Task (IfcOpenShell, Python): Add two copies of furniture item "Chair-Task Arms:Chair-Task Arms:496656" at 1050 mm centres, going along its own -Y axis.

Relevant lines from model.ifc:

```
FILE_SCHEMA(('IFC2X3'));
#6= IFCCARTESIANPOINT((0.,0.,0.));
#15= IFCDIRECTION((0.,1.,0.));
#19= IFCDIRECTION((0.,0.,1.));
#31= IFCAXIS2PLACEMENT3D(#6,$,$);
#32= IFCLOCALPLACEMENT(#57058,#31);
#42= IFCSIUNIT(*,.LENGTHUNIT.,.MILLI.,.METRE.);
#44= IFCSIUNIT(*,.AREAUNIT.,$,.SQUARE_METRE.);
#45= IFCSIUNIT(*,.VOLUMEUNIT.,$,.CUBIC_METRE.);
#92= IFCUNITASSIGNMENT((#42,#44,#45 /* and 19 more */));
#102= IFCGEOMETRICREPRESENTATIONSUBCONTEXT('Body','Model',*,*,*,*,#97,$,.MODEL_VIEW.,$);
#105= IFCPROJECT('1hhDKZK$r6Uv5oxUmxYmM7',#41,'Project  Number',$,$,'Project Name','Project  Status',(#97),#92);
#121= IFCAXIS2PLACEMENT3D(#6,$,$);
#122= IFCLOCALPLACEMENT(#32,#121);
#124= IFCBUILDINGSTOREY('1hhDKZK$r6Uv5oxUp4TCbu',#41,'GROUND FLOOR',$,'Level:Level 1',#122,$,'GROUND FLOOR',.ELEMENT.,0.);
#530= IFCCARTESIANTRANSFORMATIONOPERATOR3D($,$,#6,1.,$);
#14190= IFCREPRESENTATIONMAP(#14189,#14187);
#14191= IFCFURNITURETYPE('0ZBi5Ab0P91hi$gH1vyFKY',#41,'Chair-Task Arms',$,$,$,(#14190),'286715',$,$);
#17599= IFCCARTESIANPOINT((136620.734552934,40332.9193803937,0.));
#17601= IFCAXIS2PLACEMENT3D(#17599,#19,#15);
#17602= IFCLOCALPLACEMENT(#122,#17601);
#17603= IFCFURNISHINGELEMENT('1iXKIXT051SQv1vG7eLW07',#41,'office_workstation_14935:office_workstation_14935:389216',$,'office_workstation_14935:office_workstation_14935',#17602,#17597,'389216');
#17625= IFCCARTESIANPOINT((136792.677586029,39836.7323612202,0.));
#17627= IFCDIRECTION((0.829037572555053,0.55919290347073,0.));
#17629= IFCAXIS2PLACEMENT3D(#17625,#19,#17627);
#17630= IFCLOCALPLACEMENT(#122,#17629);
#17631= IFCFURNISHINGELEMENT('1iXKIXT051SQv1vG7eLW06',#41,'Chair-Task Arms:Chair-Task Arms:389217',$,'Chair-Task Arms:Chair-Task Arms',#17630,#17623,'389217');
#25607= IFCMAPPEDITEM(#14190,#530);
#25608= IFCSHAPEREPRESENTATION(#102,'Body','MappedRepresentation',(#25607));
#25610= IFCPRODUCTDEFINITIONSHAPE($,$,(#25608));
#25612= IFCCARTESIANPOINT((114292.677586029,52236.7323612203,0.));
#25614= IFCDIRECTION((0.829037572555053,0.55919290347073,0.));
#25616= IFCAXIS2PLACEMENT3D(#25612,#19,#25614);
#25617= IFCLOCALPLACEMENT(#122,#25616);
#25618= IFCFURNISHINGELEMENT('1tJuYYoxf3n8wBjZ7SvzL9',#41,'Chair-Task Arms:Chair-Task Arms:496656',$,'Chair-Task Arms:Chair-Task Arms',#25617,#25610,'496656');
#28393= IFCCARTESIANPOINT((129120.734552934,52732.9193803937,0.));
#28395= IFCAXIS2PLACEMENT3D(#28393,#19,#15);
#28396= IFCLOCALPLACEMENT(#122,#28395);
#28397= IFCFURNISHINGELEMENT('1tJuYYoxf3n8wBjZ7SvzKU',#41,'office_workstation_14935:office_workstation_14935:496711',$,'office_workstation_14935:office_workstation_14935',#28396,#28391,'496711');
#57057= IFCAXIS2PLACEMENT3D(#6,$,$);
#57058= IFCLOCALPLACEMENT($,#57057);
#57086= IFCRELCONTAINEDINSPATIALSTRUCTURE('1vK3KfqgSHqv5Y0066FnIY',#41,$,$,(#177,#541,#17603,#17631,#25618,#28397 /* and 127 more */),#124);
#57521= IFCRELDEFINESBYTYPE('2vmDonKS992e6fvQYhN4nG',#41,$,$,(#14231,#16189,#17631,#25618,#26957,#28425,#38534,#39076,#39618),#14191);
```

```python
import ifcopenshell
import ifcopenshell.api.geometry
import ifcopenshell.api.root
import ifcopenshell.util.element
import ifcopenshell.util.placement
import ifcopenshell.util.unit

model = ifcopenshell.open("model.ifc")
unit_scale = ifcopenshell.util.unit.calculate_unit_scale(model)


def reuse_history(source, copy):
    """copy_class also copies each property set's owner history, people and application; keep the originals."""
    for rel in copy.IsDefinedBy:
        if rel.is_a("IfcRelDefinesByProperties") and (history := rel.RelatingPropertyDefinition.OwnerHistory):
            rel.RelatingPropertyDefinition.OwnerHistory = source.OwnerHistory
            ifcopenshell.util.element.remove_deep2(model, history)


source = model.by_id(25618)
base = ifcopenshell.util.placement.get_local_placement(source.ObjectPlacement)
step = -base[:3, 1] * 1.05 / unit_scale

for i in range(1, 3):
    copy = ifcopenshell.api.root.copy_class(model, product=source)
    copy.Representation = ifcopenshell.util.element.copy_deep(
        model, source.Representation, exclude=["IfcGeometricRepresentationContext", "IfcRepresentationMap"]
    )
    copy.Name = "Chair-Task Arms:Chair-Task Arms"
    copy.Tag = None
    reuse_history(source, copy)
    matrix = base.copy()
    matrix[:3, 3] += i * step
    print("added at", matrix[:3, 3].round(3) + 0.0)
    ifcopenshell.api.geometry.edit_object_placement(model, product=copy, matrix=matrix, is_si=False)

model.write("model_edited.ifc")
```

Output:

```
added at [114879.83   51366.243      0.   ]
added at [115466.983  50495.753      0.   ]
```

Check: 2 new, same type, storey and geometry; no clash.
